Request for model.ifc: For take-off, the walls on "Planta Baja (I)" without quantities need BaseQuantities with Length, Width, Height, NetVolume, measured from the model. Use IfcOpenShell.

First a look at what the model holds.

```python
import ifcopenshell
import ifcopenshell.util.element
import ifcopenshell.util.unit

model = ifcopenshell.open("model.ifc")
print(model.schema)
for unit_type in ("LENGTHUNIT", "AREAUNIT", "VOLUMEUNIT"):
    print(unit_type, ifcopenshell.util.unit.calculate_unit_scale(model, unit_type))
storey = next(s for s in model.by_type("IfcBuildingStorey") if s.Name == "Planta Baja (I)")
walls = [e for e in ifcopenshell.util.element.get_decomposition(storey) if e.is_a("IfcWall")]
for e in sorted(walls, key=lambda e: e.id()):
    print(e.id(), e.is_a(), e.Name, list(ifcopenshell.util.element.get_psets(e, qtos_only=True)), sep=" | ")
```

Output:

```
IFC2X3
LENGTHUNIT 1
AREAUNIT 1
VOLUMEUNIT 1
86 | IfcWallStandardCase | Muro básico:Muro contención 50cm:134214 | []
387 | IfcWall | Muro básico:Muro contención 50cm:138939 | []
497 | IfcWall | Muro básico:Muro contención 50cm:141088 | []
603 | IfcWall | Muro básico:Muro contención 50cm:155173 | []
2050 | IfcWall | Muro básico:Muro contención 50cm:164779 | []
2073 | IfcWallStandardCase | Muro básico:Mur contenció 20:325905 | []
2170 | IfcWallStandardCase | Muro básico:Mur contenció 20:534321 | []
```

```python
import ifcopenshell
import ifcopenshell.api.pset
import ifcopenshell.geom
import ifcopenshell.util.element
import ifcopenshell.util.shape
import ifcopenshell.util.unit

model = ifcopenshell.open("model.ifc")
unit_scale = ifcopenshell.util.unit.calculate_unit_scale(model)
volume_scale = ifcopenshell.util.unit.calculate_unit_scale(model, "VOLUMEUNIT")
settings = ifcopenshell.geom.settings()

storey = next(s for s in model.by_type("IfcBuildingStorey") if s.Name == "Planta Baja (I)")
walls = [e for e in ifcopenshell.util.element.get_decomposition(storey) if e.is_a("IfcWall")]

for e in sorted(walls, key=lambda e: e.id()):
    if ifcopenshell.util.element.get_psets(e, qtos_only=True, should_inherit=False):
        continue
    # Geometry comes back in metres, in the element's own axes.
    shape = ifcopenshell.geom.create_shape(settings, e)
    values = {
        "Length": ifcopenshell.util.shape.get_x(shape.geometry) / unit_scale,
        "Width": ifcopenshell.util.shape.get_y(shape.geometry) / unit_scale,
        "Height": ifcopenshell.util.shape.get_z(shape.geometry) / unit_scale,
        "NetVolume": ifcopenshell.util.shape.get_volume(shape.geometry) / volume_scale,
    }
    qto = ifcopenshell.api.pset.add_qto(model, product=e, name="BaseQuantities")
    ifcopenshell.api.pset.edit_qto(model, qto=qto, properties=values)
    print(e.id(), {k: round(v, 3) for k, v in values.items()})

model.write("model-out.ifc")
```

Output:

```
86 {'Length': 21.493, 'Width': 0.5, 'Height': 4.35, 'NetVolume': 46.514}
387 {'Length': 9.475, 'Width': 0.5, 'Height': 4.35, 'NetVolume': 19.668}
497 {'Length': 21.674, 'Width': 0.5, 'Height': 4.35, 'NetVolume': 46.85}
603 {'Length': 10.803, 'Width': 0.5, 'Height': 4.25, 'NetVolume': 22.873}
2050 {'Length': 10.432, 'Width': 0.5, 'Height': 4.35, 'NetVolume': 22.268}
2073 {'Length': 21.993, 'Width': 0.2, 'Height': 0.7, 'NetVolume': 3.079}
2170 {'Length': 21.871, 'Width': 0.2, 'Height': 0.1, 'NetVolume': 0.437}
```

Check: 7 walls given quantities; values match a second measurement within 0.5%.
